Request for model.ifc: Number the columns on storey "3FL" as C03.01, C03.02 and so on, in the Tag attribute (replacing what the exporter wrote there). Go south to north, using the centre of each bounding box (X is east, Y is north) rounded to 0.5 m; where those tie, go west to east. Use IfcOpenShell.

First a look at what the model holds.

```python
import ifcopenshell
import ifcopenshell.util.element
import ifcopenshell.util.placement

model = ifcopenshell.open("model.ifc")
print(model.schema)
storey = next(s for s in model.by_type("IfcBuildingStorey") if s.Name == "3FL")
columns = [e for e in ifcopenshell.util.element.get_decomposition(storey) if e.is_a("IfcColumn")]
for e in sorted(columns, key=lambda e: e.id()):
    origin = ifcopenshell.util.placement.get_local_placement(e.ObjectPlacement)[:3, 3]
    print(e.id(), e.Tag, e.Name, origin.round(2) + 0.0, sep=" | ")
```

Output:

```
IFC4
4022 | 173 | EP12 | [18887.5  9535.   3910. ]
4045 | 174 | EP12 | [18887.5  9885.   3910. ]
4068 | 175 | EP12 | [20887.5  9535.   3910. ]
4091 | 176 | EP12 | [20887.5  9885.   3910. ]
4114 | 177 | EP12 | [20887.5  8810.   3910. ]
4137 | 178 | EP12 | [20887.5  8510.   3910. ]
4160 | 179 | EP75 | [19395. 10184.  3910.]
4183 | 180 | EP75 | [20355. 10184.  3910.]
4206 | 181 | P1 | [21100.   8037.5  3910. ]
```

```python
import ifcopenshell
import ifcopenshell.geom
import ifcopenshell.util.element
import ifcopenshell.util.shape

model = ifcopenshell.open("model.ifc")
settings = ifcopenshell.geom.settings()
settings.set("use-world-coords", True)


def centre(element):
    shape = ifcopenshell.geom.create_shape(settings, element)
    return ifcopenshell.util.shape.get_bbox_centroid(shape.geometry)


storey = next(s for s in model.by_type("IfcBuildingStorey") if s.Name == "3FL")
columns = [e for e in ifcopenshell.util.element.get_decomposition(storey) if e.is_a("IfcColumn")]

# Insertion points can sit at a corner or the storey origin, so sort by the geometry (in metres).
centres = {e: centre(e) for e in columns}
columns.sort(key=lambda e: (round(centres[e][1] / 0.5), centres[e][0]))

for i, e in enumerate(columns, start=1):
    number = f"C03.{i:02d}"
    e.Tag = number
    print(e.id(), number)

model.write("model_edited.ifc")
```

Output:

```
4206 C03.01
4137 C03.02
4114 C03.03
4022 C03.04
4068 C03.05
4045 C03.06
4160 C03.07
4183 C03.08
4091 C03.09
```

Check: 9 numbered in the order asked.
